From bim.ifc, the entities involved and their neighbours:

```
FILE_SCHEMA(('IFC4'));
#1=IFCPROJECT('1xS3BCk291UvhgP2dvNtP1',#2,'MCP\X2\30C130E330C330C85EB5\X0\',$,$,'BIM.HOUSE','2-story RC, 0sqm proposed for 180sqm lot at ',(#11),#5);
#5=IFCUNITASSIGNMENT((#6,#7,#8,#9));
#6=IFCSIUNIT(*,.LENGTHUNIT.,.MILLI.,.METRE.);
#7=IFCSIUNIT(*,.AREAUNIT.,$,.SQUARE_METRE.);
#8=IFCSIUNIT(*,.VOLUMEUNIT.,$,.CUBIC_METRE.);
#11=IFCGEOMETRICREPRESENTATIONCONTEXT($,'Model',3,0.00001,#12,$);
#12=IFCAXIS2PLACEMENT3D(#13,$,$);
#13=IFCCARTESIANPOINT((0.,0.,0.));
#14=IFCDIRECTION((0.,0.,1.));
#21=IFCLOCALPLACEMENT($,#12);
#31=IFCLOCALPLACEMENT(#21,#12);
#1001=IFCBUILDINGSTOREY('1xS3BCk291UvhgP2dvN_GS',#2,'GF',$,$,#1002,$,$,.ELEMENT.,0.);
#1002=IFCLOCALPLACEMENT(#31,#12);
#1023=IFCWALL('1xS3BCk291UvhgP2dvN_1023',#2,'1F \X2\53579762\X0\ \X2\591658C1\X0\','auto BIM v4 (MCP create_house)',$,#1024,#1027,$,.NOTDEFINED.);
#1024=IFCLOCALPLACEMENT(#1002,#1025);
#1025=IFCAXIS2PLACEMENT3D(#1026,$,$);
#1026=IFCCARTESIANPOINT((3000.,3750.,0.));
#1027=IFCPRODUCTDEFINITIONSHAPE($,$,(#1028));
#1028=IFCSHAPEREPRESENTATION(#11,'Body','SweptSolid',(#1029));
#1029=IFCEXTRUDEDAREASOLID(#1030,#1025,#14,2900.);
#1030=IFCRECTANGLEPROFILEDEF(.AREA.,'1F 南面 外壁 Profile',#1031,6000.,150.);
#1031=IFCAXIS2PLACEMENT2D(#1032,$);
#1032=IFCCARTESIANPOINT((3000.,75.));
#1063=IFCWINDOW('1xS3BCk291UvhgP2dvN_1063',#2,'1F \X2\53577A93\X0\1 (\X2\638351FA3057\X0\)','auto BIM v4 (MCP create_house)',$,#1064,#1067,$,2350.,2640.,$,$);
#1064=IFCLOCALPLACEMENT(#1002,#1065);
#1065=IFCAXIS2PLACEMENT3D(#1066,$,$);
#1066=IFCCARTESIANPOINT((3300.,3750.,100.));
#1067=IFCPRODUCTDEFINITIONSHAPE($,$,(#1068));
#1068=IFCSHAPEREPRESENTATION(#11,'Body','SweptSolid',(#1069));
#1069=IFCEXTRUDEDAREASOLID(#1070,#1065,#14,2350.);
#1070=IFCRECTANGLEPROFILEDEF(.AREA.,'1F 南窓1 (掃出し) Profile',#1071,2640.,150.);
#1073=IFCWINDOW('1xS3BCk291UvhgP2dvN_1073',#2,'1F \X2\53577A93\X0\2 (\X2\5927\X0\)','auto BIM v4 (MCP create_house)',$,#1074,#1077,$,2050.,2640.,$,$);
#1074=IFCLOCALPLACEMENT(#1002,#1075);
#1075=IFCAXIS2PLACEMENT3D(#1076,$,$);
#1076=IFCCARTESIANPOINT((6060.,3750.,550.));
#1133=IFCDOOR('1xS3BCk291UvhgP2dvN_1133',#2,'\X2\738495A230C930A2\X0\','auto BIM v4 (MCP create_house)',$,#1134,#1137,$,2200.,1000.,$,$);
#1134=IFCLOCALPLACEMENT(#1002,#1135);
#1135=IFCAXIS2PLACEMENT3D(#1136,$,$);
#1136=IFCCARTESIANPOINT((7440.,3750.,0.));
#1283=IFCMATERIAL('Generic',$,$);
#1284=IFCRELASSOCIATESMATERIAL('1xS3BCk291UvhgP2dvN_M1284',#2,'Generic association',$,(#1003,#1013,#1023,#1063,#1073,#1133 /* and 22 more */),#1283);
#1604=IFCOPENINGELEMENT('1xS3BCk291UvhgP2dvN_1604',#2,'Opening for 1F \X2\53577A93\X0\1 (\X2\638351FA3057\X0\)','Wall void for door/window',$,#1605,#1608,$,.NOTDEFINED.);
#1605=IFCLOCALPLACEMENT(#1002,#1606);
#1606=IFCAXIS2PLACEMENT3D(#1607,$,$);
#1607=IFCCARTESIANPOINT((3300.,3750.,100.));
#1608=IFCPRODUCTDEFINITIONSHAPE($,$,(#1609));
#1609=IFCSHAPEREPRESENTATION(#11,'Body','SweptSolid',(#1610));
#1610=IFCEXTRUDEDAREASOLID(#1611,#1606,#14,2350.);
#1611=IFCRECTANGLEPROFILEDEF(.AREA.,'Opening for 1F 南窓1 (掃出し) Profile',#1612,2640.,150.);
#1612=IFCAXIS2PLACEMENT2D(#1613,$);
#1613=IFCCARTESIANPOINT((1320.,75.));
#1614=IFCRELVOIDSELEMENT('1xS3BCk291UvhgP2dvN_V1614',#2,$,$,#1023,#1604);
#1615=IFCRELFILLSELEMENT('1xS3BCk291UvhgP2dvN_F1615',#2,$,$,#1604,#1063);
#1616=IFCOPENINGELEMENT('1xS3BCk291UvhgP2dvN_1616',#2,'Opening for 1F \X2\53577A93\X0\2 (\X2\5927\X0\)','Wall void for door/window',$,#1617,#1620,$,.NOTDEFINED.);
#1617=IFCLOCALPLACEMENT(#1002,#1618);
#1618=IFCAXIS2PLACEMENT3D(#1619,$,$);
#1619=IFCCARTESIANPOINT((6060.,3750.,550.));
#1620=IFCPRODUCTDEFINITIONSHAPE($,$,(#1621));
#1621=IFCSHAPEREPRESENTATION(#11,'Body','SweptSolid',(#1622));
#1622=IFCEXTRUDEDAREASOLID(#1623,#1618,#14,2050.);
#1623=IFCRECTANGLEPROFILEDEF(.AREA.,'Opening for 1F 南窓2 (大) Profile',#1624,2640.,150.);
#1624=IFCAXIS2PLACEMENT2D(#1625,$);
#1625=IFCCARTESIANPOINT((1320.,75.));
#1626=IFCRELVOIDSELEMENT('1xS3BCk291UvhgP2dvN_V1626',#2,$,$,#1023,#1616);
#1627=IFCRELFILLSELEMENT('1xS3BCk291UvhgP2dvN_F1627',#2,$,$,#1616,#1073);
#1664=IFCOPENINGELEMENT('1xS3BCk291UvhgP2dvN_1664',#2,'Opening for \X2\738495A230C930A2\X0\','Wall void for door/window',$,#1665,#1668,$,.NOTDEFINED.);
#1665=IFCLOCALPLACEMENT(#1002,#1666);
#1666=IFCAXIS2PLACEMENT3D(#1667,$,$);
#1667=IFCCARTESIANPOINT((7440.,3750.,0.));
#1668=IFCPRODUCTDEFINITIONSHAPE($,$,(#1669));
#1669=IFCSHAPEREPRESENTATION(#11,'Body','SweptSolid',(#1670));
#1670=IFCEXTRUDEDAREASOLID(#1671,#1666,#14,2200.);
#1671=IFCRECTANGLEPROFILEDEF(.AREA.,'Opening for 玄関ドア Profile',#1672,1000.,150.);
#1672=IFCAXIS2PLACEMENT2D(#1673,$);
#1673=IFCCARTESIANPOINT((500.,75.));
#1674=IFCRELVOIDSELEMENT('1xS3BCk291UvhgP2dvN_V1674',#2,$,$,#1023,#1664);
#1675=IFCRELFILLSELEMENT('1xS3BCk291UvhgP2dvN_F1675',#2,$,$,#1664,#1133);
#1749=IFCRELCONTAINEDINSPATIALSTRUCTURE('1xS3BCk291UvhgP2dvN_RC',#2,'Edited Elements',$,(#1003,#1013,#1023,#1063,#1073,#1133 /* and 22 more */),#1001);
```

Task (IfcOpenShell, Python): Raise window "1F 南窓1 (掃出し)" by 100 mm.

```python
import numpy as np
import ifcopenshell
import ifcopenshell.api.geometry
import ifcopenshell.util.placement
import ifcopenshell.util.unit

model = ifcopenshell.open("bim.ifc")
unit_scale = ifcopenshell.util.unit.calculate_unit_scale(model)

window = model.by_guid("1xS3BCk291UvhgP2dvN_1063")
opening = window.FillsVoids[0].RelatingOpeningElement
dz = 100.0

shift = np.array([0.0, 0.0, dz])
# The window is not placed relative to its opening, so move both.
for product in (opening, window):
    matrix = ifcopenshell.util.placement.get_local_placement(product.ObjectPlacement)
    matrix[:3, 3] += shift
    ifcopenshell.api.geometry.edit_object_placement(model, product=product, matrix=matrix, is_si=False)

print(f"moved by {dz * unit_scale:+.3f} m")

model.write("bim_updated.ifc")
```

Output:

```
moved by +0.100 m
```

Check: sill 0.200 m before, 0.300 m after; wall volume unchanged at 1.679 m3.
